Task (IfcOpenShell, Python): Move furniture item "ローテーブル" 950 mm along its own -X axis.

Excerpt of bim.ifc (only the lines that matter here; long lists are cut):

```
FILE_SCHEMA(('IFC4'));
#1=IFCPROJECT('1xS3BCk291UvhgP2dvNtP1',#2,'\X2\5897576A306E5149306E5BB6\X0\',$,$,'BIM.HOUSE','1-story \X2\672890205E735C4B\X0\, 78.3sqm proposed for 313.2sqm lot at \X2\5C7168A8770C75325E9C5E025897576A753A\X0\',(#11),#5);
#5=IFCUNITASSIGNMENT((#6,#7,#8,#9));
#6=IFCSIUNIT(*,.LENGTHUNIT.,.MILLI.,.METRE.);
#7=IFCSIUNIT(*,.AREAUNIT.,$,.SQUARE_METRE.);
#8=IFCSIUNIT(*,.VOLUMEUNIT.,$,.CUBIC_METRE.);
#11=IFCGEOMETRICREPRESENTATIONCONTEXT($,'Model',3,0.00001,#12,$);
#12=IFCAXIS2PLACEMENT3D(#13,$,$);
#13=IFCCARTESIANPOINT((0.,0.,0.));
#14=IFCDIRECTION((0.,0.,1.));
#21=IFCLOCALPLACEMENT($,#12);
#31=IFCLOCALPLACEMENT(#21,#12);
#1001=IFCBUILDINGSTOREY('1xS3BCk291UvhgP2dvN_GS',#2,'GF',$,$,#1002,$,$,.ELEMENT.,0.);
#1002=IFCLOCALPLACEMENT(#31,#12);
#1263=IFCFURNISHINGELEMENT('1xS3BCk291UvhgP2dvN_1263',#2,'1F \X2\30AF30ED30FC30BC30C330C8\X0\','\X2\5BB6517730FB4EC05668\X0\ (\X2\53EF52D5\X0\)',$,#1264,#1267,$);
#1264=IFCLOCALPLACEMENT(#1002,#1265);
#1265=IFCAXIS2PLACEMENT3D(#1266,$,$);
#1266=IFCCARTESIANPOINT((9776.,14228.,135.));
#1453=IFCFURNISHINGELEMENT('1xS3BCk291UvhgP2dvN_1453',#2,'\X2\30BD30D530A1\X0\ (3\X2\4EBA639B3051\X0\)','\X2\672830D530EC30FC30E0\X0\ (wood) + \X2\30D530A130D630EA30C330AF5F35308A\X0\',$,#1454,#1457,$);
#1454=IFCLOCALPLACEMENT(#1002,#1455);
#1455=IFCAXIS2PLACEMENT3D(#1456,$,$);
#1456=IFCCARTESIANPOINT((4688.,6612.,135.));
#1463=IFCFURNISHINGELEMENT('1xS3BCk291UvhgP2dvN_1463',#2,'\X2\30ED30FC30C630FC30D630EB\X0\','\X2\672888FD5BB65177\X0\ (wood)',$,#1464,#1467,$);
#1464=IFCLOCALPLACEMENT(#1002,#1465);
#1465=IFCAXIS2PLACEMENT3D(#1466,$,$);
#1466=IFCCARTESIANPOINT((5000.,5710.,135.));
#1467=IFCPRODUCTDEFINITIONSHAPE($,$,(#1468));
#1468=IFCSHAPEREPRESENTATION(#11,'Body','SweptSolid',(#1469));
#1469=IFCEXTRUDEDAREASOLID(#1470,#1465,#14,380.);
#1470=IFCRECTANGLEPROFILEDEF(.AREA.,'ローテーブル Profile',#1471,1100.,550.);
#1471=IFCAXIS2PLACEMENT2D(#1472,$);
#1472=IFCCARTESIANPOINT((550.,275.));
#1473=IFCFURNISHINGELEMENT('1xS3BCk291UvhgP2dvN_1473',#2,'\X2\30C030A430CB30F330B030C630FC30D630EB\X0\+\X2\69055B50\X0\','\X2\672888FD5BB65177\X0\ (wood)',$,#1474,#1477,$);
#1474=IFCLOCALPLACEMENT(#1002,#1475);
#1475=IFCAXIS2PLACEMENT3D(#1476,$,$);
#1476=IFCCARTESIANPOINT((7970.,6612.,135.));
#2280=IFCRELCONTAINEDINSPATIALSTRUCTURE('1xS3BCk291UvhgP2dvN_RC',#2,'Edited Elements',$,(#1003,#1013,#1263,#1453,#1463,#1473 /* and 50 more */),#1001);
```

```python
import ifcopenshell
import ifcopenshell.api.geometry
import ifcopenshell.util.placement

model = ifcopenshell.open("bim.ifc")

item = model.by_id(1463)
matrix = ifcopenshell.util.placement.get_local_placement(item.ObjectPlacement)
matrix[:3, 3] -= matrix[:3, 0] * 950.0
ifcopenshell.api.geometry.edit_object_placement(model, product=item, matrix=matrix, is_si=False)

print(ifcopenshell.util.placement.get_local_placement(item.ObjectPlacement).round(3) + 0.0)

model.write("bim-out.ifc")
```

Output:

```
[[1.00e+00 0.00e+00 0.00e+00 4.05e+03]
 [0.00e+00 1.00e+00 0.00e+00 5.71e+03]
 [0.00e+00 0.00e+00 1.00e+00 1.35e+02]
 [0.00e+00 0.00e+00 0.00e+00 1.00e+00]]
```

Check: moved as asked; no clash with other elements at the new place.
